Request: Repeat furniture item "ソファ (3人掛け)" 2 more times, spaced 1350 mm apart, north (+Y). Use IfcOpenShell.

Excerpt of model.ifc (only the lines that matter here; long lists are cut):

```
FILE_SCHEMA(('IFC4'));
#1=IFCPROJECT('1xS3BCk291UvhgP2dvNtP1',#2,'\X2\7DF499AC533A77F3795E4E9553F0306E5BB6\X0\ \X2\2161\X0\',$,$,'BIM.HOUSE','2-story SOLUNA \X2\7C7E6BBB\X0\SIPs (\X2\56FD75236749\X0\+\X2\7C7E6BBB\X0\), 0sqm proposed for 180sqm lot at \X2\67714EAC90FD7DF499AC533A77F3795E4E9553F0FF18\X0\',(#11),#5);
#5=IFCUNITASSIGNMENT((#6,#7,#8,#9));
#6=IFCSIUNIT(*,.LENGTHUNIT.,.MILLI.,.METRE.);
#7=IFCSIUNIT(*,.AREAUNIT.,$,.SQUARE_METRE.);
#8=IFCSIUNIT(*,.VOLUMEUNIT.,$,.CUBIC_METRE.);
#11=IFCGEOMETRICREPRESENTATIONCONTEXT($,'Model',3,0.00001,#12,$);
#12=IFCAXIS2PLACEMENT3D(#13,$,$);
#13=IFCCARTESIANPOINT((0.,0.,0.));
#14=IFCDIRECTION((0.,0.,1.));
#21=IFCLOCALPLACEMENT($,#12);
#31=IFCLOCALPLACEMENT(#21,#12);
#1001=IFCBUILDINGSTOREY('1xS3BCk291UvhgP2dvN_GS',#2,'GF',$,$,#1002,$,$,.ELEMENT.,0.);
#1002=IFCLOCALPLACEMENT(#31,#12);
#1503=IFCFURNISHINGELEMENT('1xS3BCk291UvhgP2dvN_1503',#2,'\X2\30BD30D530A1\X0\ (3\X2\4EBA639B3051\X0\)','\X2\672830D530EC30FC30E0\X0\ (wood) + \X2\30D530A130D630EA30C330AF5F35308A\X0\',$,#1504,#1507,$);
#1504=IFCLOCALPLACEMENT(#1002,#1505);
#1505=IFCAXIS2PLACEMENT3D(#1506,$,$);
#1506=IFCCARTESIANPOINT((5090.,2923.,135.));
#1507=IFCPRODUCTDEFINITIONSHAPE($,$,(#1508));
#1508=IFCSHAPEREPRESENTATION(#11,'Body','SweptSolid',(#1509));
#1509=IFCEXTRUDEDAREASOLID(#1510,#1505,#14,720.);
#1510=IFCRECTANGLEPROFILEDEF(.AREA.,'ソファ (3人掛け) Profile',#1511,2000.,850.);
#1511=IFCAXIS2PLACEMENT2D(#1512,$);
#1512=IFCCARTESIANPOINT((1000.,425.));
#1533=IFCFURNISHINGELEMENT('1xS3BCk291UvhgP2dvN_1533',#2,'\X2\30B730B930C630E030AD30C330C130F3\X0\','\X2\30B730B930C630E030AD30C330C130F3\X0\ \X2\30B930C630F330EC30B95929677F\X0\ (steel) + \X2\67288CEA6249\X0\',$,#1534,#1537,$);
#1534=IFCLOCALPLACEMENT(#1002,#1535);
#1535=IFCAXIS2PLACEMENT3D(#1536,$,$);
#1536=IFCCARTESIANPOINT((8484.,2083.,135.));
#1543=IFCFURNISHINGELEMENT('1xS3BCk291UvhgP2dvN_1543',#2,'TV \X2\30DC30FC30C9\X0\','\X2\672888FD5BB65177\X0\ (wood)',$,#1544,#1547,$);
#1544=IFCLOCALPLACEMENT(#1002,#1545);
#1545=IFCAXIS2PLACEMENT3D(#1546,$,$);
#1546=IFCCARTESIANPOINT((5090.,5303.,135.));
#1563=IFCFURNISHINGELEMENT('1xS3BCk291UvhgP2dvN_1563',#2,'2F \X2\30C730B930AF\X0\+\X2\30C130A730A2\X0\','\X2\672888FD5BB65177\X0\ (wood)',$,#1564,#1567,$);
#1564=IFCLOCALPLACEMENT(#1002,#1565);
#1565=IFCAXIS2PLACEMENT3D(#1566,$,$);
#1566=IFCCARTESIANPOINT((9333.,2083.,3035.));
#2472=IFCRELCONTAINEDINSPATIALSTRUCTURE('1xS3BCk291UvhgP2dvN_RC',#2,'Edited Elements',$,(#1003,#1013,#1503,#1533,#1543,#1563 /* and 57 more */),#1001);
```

```python
import numpy as np
import ifcopenshell
import ifcopenshell.api.geometry
import ifcopenshell.api.root
import ifcopenshell.util.element
import ifcopenshell.util.placement
import ifcopenshell.util.unit

model = ifcopenshell.open("model.ifc")
unit_scale = ifcopenshell.util.unit.calculate_unit_scale(model)


def reuse_history(source, copy):
    """copy_class also copies each property set's owner history, people and application; keep the originals."""
    for rel in copy.IsDefinedBy:
        if rel.is_a("IfcRelDefinesByProperties") and (history := rel.RelatingPropertyDefinition.OwnerHistory):
            rel.RelatingPropertyDefinition.OwnerHistory = source.OwnerHistory
            ifcopenshell.util.element.remove_deep2(model, history)


source = model.by_guid("1xS3BCk291UvhgP2dvN_1503")
base = ifcopenshell.util.placement.get_local_placement(source.ObjectPlacement)
step = np.array([0.0, 1.0, 0.0]) * 1.35 / unit_scale

for i in range(1, 3):
    copy = ifcopenshell.api.root.copy_class(model, product=source)
    copy.Representation = ifcopenshell.util.element.copy_deep(
        model, source.Representation, exclude=["IfcGeometricRepresentationContext", "IfcRepresentationMap"]
    )
    reuse_history(source, copy)
    matrix = base.copy()
    matrix[:3, 3] += i * step
    print("added at", matrix[:3, 3].round(3) + 0.0)
    ifcopenshell.api.geometry.edit_object_placement(model, product=copy, matrix=matrix, is_si=False)

model.write("model_v2.ifc")
```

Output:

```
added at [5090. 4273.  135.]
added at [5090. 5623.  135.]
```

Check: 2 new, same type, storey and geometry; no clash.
